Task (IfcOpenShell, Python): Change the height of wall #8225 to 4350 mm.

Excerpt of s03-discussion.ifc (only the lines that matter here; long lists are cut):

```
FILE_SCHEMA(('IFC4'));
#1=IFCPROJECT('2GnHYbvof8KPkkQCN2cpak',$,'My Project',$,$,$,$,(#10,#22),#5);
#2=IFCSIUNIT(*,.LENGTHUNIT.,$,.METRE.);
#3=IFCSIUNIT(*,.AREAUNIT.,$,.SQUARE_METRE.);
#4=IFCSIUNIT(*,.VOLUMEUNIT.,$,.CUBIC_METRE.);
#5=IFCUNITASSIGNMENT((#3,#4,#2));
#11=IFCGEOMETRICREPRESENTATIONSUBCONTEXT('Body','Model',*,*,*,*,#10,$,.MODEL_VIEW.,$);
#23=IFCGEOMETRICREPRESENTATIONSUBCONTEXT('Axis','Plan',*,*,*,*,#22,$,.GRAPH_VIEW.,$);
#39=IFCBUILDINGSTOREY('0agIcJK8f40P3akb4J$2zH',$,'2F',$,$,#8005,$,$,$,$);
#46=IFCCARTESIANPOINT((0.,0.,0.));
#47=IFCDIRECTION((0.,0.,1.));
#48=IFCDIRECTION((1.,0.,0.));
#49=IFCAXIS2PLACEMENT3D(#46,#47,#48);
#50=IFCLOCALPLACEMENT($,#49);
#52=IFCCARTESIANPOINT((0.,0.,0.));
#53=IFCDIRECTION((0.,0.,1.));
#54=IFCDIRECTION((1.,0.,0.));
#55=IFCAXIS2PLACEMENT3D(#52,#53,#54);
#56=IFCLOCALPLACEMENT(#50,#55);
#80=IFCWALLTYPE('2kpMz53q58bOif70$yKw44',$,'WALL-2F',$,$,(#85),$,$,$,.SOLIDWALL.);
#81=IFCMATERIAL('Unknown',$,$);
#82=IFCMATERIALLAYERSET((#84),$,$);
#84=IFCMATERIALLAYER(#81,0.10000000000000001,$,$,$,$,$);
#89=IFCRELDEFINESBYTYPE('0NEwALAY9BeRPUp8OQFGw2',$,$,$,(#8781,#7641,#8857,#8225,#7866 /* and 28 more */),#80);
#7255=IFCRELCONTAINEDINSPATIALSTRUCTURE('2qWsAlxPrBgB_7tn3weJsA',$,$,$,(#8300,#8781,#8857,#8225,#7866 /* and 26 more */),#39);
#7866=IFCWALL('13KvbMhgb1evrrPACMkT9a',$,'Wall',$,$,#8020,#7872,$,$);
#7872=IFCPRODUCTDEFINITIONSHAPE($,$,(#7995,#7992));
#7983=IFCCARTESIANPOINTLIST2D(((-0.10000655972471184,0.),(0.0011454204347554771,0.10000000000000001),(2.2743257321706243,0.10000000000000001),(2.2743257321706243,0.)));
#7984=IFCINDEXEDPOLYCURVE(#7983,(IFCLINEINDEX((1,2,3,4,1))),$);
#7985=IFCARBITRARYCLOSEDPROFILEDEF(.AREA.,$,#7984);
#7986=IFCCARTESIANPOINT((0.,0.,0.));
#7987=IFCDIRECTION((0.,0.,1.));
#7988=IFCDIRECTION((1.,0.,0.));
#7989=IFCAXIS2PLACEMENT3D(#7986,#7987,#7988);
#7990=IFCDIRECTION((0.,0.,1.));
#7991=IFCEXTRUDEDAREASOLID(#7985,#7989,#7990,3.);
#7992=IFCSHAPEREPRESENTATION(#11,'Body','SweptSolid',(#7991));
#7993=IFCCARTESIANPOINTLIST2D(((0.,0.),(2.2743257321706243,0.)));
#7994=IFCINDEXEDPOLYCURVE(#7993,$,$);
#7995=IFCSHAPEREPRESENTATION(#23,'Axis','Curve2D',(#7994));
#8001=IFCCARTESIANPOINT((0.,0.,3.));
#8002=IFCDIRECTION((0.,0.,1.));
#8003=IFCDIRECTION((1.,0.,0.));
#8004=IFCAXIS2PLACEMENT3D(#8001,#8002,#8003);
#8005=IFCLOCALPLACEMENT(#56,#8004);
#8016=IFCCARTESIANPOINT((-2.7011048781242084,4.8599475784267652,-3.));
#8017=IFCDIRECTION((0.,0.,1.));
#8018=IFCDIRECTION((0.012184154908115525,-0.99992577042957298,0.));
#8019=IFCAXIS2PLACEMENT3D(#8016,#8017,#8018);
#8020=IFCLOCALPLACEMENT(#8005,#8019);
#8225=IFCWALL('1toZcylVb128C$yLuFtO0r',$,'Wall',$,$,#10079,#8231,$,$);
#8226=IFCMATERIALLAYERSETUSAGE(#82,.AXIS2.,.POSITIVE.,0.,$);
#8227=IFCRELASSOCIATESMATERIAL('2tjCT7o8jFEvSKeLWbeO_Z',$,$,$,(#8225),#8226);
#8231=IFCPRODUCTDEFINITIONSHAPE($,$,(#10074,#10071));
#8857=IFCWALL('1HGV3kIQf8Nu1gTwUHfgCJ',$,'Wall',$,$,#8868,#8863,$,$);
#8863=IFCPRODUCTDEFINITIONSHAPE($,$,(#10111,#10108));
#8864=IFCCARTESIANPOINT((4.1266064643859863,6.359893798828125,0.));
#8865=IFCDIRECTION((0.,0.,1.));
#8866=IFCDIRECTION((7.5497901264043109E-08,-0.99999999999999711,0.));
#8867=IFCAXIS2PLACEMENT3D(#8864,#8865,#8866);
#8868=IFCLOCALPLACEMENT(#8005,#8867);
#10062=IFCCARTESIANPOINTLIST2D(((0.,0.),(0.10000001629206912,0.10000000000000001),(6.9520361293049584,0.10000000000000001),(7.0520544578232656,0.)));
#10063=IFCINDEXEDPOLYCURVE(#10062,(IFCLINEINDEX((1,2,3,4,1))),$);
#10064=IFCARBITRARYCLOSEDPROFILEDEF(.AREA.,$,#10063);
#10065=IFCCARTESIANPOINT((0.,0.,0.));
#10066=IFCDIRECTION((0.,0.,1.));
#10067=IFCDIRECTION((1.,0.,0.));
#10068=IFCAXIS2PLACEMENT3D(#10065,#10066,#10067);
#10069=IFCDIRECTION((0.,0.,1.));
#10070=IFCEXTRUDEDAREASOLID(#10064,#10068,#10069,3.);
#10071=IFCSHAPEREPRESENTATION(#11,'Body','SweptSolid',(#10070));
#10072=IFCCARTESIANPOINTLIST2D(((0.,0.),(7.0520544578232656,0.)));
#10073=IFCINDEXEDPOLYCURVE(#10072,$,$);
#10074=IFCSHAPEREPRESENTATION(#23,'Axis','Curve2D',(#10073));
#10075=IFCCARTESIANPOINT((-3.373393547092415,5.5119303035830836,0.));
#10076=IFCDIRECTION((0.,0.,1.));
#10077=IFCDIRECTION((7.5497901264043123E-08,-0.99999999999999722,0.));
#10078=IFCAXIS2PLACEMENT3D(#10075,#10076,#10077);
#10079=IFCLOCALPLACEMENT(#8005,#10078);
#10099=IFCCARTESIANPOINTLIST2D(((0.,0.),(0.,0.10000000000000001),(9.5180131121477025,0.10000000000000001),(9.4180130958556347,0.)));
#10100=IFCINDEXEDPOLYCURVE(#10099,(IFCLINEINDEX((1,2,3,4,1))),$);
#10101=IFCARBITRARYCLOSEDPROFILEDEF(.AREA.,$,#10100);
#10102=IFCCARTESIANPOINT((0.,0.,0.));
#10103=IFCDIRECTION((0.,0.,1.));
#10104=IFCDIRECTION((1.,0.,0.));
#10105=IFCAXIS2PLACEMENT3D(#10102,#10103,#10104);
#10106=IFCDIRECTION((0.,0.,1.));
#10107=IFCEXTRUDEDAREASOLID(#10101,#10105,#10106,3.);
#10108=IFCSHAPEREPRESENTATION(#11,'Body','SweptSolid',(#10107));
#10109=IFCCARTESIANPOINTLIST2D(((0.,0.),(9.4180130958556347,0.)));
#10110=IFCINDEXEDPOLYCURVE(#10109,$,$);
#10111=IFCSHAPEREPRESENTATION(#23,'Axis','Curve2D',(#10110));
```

```python
import ifcopenshell
import ifcopenshell.geom
import ifcopenshell.util.representation
import ifcopenshell.util.shape
import ifcopenshell.util.unit

model = ifcopenshell.open("s03-discussion.ifc")
unit_scale = ifcopenshell.util.unit.calculate_unit_scale(model)
settings = ifcopenshell.geom.settings()


def volume(element):
    """Net volume in cubic metres, openings subtracted."""
    shape = ifcopenshell.geom.create_shape(settings, element)
    return ifcopenshell.util.shape.get_volume(shape.geometry)


wall = model.by_id(8225)
before = volume(wall)

body = ifcopenshell.util.representation.get_representation(wall, "Model", "Body")
solid = body.Items[0]
old_height = solid.Depth
solid.Depth = 4.35 / unit_scale
after = volume(wall)

print(f"height {old_height:g} -> {solid.Depth:g}, volume {before:.3f} -> {after:.3f} m3")

model.write("s03-discussion_rev.ifc")
```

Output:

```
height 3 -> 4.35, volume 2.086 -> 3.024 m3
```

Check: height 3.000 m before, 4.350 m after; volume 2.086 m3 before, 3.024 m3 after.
